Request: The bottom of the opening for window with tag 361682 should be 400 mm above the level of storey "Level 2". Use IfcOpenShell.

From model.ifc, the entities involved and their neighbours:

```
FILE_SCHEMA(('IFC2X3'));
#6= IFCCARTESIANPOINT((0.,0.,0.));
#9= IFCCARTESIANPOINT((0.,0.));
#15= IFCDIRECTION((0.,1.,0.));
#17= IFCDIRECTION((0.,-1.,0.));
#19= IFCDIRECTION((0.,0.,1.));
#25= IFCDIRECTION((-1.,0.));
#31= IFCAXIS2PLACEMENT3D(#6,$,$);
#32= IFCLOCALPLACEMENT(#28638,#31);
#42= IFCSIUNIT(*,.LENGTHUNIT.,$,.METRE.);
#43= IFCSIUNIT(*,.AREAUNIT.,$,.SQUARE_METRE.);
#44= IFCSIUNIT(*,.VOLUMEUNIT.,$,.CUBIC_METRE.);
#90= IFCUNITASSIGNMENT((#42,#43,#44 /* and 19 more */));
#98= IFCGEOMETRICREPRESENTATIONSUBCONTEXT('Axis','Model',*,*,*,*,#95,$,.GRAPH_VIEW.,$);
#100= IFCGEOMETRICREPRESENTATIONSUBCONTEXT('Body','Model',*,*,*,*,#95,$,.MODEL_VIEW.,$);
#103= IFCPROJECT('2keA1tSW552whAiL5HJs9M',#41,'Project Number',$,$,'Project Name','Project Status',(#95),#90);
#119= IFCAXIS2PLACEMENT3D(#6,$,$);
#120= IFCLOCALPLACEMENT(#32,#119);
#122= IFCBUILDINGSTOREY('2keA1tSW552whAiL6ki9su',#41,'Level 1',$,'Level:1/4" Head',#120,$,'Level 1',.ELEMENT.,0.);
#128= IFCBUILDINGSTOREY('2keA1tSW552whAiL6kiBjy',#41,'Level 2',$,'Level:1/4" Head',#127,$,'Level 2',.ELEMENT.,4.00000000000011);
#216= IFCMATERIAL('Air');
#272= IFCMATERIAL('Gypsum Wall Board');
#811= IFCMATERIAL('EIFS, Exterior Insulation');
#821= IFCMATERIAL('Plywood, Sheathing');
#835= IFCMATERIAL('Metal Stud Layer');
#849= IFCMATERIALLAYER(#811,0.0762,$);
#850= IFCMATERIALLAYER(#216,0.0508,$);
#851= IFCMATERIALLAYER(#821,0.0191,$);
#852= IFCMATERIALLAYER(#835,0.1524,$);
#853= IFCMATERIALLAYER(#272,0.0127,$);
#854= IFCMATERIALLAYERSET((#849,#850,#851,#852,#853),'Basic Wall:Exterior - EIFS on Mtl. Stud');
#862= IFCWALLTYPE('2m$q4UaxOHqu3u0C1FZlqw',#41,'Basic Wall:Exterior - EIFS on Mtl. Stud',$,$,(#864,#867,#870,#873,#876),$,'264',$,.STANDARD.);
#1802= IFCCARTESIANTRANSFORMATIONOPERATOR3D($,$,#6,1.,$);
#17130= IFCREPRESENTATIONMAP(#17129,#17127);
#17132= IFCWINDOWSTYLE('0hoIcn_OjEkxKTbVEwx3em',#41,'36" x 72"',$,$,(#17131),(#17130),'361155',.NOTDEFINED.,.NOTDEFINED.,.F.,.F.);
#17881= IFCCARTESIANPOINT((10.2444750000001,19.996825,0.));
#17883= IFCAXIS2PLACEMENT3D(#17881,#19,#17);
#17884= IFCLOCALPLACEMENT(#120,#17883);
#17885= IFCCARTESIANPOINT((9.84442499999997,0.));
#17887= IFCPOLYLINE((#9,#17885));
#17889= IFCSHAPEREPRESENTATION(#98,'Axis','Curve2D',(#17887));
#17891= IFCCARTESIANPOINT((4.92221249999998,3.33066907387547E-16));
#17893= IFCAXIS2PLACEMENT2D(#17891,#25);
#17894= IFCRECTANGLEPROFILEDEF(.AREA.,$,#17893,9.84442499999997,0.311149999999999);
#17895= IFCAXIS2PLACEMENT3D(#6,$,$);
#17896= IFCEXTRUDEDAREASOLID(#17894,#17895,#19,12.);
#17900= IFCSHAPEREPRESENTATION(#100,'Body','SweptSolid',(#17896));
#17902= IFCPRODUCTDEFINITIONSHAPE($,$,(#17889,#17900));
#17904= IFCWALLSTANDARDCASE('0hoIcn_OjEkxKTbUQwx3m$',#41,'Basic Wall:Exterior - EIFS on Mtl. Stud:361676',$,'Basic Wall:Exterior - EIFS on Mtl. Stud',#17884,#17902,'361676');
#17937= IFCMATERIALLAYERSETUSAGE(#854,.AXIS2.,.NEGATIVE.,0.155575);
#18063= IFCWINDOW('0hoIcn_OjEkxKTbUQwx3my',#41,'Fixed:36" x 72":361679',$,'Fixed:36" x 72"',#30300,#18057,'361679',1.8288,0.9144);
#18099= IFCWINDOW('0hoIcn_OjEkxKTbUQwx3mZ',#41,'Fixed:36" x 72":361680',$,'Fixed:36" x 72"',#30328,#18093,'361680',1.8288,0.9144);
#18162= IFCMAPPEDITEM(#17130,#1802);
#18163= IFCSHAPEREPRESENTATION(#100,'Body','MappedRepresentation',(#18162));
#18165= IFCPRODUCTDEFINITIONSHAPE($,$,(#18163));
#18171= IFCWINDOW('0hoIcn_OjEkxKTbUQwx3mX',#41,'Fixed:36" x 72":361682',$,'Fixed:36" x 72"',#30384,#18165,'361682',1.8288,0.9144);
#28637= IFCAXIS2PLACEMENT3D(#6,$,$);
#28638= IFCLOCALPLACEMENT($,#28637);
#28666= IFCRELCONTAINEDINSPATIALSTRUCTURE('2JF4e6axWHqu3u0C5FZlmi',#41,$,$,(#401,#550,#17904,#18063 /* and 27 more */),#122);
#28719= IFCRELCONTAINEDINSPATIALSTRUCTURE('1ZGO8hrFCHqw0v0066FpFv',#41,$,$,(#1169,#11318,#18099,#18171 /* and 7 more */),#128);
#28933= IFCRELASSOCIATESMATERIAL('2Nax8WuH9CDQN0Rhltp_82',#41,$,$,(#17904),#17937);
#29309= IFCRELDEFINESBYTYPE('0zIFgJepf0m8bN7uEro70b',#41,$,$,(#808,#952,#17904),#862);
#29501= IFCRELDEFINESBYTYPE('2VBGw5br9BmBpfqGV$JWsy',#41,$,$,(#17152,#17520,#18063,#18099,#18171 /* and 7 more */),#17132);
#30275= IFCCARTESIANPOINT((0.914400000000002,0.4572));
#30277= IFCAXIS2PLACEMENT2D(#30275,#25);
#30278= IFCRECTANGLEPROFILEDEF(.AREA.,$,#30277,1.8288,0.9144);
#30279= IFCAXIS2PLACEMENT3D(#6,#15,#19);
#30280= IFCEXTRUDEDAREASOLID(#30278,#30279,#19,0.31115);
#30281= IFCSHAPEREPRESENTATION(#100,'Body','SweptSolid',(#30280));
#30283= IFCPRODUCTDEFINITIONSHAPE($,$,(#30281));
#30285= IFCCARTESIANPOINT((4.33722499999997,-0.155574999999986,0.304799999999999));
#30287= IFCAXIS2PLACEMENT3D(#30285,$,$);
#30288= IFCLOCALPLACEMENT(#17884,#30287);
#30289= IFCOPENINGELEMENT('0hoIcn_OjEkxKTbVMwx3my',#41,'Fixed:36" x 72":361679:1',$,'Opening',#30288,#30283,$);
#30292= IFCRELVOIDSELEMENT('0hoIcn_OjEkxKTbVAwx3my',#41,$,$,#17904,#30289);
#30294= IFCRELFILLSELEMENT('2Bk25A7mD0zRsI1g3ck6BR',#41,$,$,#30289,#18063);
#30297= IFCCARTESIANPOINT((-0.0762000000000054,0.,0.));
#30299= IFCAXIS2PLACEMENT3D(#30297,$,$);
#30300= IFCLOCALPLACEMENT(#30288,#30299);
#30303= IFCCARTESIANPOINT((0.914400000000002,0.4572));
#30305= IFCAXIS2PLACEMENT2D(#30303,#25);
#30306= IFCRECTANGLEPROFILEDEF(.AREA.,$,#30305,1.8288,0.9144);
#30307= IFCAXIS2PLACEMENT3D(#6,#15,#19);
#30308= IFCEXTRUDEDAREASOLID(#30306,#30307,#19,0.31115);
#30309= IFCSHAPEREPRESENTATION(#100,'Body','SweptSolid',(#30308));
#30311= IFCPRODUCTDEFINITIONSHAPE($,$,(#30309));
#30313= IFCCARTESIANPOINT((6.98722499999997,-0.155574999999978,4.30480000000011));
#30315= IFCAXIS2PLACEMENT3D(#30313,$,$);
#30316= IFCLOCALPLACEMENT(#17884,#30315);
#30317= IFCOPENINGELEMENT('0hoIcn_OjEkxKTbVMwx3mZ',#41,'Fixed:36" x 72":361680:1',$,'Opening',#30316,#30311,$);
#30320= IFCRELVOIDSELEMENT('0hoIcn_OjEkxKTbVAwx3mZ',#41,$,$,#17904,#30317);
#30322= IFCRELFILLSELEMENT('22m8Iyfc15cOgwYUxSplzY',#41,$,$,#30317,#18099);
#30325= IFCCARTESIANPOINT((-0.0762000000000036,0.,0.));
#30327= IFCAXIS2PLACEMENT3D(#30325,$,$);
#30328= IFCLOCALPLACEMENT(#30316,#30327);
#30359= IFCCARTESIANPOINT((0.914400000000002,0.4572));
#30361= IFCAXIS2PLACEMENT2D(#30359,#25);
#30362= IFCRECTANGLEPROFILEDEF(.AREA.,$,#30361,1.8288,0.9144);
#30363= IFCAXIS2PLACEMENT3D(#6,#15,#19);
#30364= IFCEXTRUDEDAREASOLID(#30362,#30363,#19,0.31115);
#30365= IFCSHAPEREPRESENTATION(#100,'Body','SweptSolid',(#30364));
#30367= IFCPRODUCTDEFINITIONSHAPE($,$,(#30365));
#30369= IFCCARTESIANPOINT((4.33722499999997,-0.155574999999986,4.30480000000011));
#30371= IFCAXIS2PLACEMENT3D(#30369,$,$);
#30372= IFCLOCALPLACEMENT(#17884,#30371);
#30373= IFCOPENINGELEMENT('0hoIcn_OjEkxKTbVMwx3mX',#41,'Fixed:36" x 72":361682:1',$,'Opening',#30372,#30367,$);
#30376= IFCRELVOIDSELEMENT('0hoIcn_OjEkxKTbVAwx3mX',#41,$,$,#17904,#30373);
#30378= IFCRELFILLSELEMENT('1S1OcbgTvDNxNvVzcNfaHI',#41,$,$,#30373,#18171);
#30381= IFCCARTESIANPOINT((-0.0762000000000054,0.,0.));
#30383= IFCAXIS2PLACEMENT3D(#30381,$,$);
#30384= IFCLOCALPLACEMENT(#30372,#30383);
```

```python
import numpy as np
import ifcopenshell
import ifcopenshell.api.geometry
import ifcopenshell.geom
import ifcopenshell.util.element
import ifcopenshell.util.placement
import ifcopenshell.util.shape
import ifcopenshell.util.unit

model = ifcopenshell.open("model.ifc")
unit_scale = ifcopenshell.util.unit.calculate_unit_scale(model)

window = model.by_guid("0hoIcn_OjEkxKTbUQwx3mX")
opening = window.FillsVoids[0].RelatingOpeningElement
storey = ifcopenshell.util.element.get_container(window, ifc_class="IfcBuildingStorey")
level = ifcopenshell.util.placement.get_local_placement(storey.ObjectPlacement)[2, 3]

# The opening's origin need not be at the sill, so measure its lowest point.
shape = ifcopenshell.geom.create_shape(ifcopenshell.geom.settings(), opening)
bottom = ifcopenshell.util.shape.get_shape_bottom_elevation(shape, shape.geometry) / unit_scale
dz = level + 0.4 - bottom

shift = np.array([0.0, 0.0, dz])
# The window is placed relative to its opening, so it follows when the opening moves.
matrix = ifcopenshell.util.placement.get_local_placement(opening.ObjectPlacement)
matrix[:3, 3] += shift
ifcopenshell.api.geometry.edit_object_placement(
    model, product=opening, matrix=matrix, is_si=False, should_transform_children=True
)

print(f"moved by {dz * unit_scale:+.3f} m")

model.write("model_edited.ifc")
```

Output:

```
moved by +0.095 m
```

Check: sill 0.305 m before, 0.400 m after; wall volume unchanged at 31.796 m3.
